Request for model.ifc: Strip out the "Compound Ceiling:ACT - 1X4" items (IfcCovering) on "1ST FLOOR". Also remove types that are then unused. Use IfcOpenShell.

First a look at what the model holds.

```python
import ifcopenshell
import ifcopenshell.util.element

model = ifcopenshell.open("model.ifc")
print(model.schema)
storey = next(s for s in model.by_type("IfcBuildingStorey") if s.Name == "1ST FLOOR")
coverings = [e for e in ifcopenshell.util.element.get_decomposition(storey) if e.is_a("IfcCovering")]
seen = {}
for e in coverings:
    element_type = ifcopenshell.util.element.get_type(e)
    name = element_type.Name if element_type not in (None, e) else None
    seen[name] = seen.get(name, 0) + 1
for name, count in sorted(seen.items(), key=str):
    print(count, "x", name)
```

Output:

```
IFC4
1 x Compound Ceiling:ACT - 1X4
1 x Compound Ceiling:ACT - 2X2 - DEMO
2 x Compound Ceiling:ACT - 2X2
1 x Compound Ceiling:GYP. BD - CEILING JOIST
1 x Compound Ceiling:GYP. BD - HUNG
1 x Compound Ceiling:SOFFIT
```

```python
import ifcopenshell
import ifcopenshell.api.root
import ifcopenshell.util.element

model = ifcopenshell.open("model.ifc")

storey = next(s for s in model.by_type("IfcBuildingStorey") if s.Name == "1ST FLOOR")
coverings = [e for e in ifcopenshell.util.element.get_decomposition(storey) if e.is_a("IfcCovering")]
targets = [e for e in coverings if (t := ifcopenshell.util.element.get_type(e)) not in (None, e) and t.Name == "Compound Ceiling:ACT - 1X4"]
types = {ifcopenshell.util.element.get_type(e) for e in targets} - {None, *targets}

for e in targets:
    ifcopenshell.api.root.remove_product(model, product=e)
print(len(targets), "removed")

unused = [t for t in types if not ifcopenshell.util.element.get_types(t)]
for t in unused:
    ifcopenshell.api.root.remove_product(model, product=t)
print(len(unused), "unused types removed")

model.write("model-out.ifc")
```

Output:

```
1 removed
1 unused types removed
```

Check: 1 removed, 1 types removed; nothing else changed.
